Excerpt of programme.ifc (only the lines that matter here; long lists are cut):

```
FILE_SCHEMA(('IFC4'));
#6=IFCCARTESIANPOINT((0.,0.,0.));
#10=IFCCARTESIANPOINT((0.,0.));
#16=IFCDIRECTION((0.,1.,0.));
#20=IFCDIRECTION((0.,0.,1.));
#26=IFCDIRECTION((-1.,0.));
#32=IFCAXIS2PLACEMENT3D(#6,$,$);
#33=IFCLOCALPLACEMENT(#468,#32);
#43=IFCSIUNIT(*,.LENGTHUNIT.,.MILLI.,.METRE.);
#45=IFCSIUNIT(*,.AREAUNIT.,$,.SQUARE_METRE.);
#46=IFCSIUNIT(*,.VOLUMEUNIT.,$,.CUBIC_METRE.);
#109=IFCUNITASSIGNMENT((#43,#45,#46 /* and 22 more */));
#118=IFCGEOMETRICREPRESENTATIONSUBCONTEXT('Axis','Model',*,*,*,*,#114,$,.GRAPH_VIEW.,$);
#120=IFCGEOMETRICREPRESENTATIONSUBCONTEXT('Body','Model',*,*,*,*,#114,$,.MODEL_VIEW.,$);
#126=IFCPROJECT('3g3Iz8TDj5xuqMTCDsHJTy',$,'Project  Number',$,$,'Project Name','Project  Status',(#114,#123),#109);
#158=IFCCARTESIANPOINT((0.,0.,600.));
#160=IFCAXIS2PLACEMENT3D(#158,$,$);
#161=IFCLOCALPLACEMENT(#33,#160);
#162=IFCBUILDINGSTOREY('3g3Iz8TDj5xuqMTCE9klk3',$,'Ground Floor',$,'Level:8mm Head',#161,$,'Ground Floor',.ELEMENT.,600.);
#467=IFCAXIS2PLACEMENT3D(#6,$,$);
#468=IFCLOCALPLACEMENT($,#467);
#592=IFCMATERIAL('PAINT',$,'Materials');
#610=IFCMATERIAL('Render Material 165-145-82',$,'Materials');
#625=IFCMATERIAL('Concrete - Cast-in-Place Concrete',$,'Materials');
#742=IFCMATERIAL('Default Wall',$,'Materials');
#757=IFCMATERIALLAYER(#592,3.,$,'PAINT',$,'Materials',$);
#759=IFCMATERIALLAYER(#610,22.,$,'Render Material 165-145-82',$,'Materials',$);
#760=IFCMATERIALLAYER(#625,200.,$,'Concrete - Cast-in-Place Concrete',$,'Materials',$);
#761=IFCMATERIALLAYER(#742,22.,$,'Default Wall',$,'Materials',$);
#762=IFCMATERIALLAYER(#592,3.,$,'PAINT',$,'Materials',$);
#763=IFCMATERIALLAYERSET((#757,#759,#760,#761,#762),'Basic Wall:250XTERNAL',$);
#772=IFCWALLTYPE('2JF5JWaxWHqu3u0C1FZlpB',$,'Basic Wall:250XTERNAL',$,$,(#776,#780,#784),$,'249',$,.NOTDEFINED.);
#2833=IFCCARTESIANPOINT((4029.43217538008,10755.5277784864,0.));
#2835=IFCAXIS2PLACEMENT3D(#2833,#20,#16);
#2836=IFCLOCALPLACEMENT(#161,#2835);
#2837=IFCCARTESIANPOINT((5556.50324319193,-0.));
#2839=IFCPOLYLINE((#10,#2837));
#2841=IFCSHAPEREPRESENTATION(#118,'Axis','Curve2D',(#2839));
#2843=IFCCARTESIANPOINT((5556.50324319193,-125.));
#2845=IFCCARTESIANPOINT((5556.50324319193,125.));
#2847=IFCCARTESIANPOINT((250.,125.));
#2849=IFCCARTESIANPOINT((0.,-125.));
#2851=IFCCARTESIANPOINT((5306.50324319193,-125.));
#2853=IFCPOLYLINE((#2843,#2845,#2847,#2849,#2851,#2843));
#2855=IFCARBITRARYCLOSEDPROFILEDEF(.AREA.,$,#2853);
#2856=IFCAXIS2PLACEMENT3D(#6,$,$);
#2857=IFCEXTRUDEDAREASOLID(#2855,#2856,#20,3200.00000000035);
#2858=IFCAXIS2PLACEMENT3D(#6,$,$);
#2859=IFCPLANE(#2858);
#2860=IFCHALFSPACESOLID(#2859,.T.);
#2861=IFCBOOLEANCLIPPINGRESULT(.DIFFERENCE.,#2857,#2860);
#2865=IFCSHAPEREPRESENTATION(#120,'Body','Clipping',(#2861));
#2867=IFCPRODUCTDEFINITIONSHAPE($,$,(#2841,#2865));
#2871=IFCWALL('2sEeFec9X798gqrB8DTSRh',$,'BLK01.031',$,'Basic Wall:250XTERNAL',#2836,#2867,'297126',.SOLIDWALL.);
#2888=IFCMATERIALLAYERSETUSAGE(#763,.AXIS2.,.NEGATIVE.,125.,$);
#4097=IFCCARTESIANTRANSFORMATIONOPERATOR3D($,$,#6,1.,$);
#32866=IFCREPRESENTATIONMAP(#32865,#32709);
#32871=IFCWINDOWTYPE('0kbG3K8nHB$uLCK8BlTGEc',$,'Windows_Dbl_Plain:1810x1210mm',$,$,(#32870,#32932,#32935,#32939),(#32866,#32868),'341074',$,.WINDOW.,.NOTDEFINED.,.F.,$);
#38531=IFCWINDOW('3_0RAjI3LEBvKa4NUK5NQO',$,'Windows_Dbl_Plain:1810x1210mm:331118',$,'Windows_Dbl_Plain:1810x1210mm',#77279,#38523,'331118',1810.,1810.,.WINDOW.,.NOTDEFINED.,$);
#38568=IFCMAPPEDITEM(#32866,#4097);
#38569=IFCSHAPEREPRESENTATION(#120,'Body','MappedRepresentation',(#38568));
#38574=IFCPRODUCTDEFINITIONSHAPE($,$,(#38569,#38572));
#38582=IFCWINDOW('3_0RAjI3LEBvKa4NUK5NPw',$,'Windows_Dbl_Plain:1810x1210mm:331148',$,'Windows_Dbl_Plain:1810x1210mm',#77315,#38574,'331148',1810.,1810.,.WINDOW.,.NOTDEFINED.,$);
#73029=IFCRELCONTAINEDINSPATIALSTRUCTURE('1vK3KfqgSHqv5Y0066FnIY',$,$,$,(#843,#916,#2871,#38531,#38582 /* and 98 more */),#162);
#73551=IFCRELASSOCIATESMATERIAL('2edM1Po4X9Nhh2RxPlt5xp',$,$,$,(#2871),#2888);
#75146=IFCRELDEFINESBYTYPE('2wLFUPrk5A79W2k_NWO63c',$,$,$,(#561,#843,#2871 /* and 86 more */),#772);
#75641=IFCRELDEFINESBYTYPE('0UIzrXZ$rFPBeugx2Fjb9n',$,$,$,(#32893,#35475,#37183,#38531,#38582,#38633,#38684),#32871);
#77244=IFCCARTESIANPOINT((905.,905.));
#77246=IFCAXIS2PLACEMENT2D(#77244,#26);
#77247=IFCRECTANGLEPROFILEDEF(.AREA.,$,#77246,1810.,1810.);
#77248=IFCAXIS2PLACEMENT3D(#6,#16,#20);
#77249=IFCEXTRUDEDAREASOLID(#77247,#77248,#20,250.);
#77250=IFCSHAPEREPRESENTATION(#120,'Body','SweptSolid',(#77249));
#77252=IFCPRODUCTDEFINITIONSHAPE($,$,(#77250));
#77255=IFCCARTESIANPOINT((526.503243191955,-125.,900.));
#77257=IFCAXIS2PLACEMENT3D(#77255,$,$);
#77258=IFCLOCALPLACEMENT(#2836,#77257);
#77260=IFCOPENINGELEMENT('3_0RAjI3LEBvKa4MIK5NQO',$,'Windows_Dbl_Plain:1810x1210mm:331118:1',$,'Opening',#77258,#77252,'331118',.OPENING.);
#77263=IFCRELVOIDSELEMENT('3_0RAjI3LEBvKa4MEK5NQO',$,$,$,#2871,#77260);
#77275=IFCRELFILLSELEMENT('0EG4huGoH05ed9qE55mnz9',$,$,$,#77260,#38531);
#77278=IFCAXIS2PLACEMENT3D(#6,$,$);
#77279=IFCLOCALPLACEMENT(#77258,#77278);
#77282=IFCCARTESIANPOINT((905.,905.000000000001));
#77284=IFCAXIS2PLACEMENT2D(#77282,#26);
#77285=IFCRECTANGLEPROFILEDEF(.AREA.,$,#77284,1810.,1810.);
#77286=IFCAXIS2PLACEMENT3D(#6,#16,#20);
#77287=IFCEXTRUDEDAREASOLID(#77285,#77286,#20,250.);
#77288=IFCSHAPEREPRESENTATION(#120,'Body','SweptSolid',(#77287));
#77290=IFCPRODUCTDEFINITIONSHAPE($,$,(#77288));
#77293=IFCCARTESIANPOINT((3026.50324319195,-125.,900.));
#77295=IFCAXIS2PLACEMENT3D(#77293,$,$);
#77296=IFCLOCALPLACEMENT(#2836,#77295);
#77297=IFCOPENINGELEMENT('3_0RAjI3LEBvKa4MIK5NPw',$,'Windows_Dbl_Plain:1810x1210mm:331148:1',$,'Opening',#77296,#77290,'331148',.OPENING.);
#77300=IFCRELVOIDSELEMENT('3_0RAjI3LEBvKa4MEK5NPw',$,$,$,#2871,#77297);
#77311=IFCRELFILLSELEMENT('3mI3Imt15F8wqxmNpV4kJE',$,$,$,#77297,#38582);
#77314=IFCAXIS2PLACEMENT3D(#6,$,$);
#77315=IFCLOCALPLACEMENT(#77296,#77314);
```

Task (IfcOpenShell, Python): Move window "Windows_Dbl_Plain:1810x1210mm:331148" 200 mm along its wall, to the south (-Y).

```python
import ifcopenshell
import ifcopenshell.api.geometry
import ifcopenshell.util.placement
import ifcopenshell.util.unit

model = ifcopenshell.open("programme.ifc")
unit_scale = ifcopenshell.util.unit.calculate_unit_scale(model)

window = model.by_guid("3_0RAjI3LEBvKa4NUK5NPw")
opening = window.FillsVoids[0].RelatingOpeningElement
wall = opening.VoidsElements[0].RelatingBuildingElement

wall_matrix = ifcopenshell.util.placement.get_local_placement(wall.ObjectPlacement)
shift = wall_matrix[:3, 0] * -0.2 / unit_scale
before = ifcopenshell.util.placement.get_local_placement(window.ObjectPlacement)[:3, 3].copy()

# The window is placed relative to its opening, so it follows when the opening moves.
matrix = ifcopenshell.util.placement.get_local_placement(opening.ObjectPlacement)
matrix[:3, 3] += shift
ifcopenshell.api.geometry.edit_object_placement(
    model, product=opening, matrix=matrix, is_si=False, should_transform_children=True
)

after = ifcopenshell.util.placement.get_local_placement(window.ObjectPlacement)[:3, 3]
print("window moved by", (after - before).round(3) + 0.0)

model.write("programme-out.ifc")
```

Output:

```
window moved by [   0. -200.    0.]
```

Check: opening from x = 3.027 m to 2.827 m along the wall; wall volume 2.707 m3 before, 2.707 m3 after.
